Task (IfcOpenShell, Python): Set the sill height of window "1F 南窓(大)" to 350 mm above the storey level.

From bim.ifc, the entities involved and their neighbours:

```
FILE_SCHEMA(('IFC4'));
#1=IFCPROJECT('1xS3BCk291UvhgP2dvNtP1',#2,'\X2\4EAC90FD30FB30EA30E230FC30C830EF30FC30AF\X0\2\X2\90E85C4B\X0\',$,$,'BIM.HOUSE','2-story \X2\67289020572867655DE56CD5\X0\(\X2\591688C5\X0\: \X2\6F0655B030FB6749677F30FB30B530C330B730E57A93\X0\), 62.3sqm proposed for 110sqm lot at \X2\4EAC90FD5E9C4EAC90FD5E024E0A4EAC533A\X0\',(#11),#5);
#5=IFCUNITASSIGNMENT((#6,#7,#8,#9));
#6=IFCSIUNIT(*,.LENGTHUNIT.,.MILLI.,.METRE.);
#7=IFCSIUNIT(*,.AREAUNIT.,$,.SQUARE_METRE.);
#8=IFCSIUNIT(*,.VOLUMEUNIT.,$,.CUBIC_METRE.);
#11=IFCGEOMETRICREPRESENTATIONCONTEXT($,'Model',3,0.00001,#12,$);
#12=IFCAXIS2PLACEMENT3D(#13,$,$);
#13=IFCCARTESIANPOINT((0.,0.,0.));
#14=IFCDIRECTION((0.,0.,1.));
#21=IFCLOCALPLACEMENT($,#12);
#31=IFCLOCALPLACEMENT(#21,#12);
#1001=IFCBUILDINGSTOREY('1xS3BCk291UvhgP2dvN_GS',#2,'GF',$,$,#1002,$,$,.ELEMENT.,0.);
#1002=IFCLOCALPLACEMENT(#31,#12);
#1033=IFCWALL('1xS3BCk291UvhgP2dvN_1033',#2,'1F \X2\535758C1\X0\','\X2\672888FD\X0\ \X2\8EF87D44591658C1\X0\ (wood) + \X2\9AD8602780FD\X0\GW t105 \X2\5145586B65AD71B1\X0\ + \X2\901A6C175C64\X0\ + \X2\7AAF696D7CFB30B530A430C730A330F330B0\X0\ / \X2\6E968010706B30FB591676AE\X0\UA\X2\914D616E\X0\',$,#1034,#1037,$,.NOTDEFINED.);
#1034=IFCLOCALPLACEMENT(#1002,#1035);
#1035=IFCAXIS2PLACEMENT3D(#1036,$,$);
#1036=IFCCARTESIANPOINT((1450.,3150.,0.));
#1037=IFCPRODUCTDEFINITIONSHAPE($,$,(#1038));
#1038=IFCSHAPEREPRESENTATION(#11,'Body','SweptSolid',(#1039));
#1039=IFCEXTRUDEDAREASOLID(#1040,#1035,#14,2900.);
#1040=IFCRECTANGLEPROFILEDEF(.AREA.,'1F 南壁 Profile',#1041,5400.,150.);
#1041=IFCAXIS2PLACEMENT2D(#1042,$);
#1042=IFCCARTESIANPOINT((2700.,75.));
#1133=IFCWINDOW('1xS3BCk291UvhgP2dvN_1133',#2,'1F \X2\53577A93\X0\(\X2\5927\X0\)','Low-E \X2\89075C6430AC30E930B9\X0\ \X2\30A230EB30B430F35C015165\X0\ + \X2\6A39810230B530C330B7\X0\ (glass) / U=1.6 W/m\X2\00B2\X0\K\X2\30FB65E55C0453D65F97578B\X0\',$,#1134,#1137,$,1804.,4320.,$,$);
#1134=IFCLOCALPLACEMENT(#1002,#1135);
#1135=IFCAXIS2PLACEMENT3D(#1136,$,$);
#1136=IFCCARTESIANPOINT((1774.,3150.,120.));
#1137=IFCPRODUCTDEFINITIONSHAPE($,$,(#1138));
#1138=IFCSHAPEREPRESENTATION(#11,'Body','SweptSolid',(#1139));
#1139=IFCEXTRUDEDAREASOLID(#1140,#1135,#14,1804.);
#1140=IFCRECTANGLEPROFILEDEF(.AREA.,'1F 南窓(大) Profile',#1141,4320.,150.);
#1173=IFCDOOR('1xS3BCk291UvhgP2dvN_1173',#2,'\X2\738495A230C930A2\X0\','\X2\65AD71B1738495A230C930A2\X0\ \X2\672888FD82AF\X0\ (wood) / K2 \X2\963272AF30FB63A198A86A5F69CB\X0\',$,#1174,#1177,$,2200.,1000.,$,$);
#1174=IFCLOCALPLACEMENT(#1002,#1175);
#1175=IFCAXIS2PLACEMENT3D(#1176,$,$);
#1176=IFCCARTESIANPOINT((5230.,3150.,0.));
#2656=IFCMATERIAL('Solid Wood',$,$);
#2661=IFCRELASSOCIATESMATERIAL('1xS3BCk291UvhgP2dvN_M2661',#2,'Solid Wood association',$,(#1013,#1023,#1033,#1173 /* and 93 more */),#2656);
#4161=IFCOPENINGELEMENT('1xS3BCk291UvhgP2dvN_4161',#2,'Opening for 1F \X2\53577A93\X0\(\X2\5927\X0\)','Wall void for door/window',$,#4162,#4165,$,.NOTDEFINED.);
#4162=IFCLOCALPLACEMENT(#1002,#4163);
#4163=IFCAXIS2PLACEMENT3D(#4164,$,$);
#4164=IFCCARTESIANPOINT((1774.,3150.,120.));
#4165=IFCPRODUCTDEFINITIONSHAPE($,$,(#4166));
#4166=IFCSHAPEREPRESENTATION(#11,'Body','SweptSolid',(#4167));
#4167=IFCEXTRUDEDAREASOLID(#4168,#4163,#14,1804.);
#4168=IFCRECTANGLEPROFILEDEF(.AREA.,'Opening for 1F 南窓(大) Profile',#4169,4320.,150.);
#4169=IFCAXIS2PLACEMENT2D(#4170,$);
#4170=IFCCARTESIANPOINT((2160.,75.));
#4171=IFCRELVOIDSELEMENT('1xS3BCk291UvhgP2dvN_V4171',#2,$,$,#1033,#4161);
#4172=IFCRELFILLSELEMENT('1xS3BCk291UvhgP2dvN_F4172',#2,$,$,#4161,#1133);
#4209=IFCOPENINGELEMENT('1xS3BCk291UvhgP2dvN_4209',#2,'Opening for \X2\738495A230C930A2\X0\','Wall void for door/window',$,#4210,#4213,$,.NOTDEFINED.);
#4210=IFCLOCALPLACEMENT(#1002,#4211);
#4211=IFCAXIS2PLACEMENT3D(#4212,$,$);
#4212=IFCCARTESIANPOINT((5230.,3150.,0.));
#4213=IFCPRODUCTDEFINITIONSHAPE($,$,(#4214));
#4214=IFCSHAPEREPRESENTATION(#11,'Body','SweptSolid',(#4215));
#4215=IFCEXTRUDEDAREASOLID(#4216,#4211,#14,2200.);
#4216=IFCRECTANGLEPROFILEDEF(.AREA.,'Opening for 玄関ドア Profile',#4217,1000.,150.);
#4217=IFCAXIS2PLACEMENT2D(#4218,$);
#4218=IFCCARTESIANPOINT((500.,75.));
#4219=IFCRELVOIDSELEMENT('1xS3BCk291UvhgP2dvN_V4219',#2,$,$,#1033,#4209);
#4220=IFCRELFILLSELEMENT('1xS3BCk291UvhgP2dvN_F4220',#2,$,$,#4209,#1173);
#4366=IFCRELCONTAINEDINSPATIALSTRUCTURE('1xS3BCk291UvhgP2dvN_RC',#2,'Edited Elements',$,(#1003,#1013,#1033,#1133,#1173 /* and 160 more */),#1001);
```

```python
import numpy as np
import ifcopenshell
import ifcopenshell.api.geometry
import ifcopenshell.geom
import ifcopenshell.util.element
import ifcopenshell.util.placement
import ifcopenshell.util.shape
import ifcopenshell.util.unit

model = ifcopenshell.open("bim.ifc")
unit_scale = ifcopenshell.util.unit.calculate_unit_scale(model)

window = model.by_guid("1xS3BCk291UvhgP2dvN_1133")
opening = window.FillsVoids[0].RelatingOpeningElement
storey = ifcopenshell.util.element.get_container(window, ifc_class="IfcBuildingStorey")
level = ifcopenshell.util.placement.get_local_placement(storey.ObjectPlacement)[2, 3]

# The opening's origin need not be at the sill, so measure its lowest point.
shape = ifcopenshell.geom.create_shape(ifcopenshell.geom.settings(), opening)
bottom = ifcopenshell.util.shape.get_shape_bottom_elevation(shape, shape.geometry) / unit_scale
dz = level + 0.35 / unit_scale - bottom

shift = np.array([0.0, 0.0, dz])
# The window is not placed relative to its opening, so move both.
for product in (opening, window):
    matrix = ifcopenshell.util.placement.get_local_placement(product.ObjectPlacement)
    matrix[:3, 3] += shift
    ifcopenshell.api.geometry.edit_object_placement(model, product=product, matrix=matrix, is_si=False)

print(f"moved by {dz * unit_scale:+.3f} m")

model.write("bim_rev.ifc")
```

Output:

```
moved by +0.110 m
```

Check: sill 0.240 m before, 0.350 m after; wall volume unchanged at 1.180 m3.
